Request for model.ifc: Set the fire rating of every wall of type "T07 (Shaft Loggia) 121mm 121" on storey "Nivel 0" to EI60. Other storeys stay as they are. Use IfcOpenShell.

First a look at what the model holds.

```python
import ifcopenshell
import ifcopenshell.util.element

model = ifcopenshell.open("model.ifc")
print(model.schema)
storey = next(s for s in model.by_type("IfcBuildingStorey") if s.Name == "Nivel 0")
walls = [e for e in ifcopenshell.util.element.get_decomposition(storey) if e.is_a("IfcWall")]
seen = {}
for e in walls:
    element_type = ifcopenshell.util.element.get_type(e)
    key = (element_type.Name if element_type != e and element_type else None, ifcopenshell.util.element.get_pset(e, "Pset_WallCommon", "FireRating"))
    seen[key] = seen.get(key, 0) + 1
for (name, value), count in sorted(seen.items(), key=str):
    print(count, "x", name, "|", value)
```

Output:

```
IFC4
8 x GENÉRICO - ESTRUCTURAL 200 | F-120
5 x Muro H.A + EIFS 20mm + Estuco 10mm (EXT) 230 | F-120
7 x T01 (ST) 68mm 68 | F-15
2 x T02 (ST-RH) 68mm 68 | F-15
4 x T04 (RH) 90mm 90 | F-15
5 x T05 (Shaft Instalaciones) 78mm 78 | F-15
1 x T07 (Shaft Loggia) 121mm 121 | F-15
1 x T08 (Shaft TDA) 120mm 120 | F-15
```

```python
import ifcopenshell
import ifcopenshell.api.pset
import ifcopenshell.util.element

model = ifcopenshell.open("model.ifc")

storey = next(s for s in model.by_type("IfcBuildingStorey") if s.Name == "Nivel 0")
walls = [e for e in ifcopenshell.util.element.get_decomposition(storey) if e.is_a("IfcWall")]

count = 0
for e in walls:
    element_type = ifcopenshell.util.element.get_type(e)
    if element_type in (None, e) or element_type.Name != "T07 (Shaft Loggia) 121mm 121":
        continue
    # add_pset returns the element's existing set when there is one.
    pset = ifcopenshell.api.pset.add_pset(model, product=e, name="Pset_WallCommon")
    ifcopenshell.api.pset.edit_pset(model, pset=pset, properties={"FireRating": "EI60"})
    count += 1

print(count, "walls updated")

model.write("model_updated.ifc")
```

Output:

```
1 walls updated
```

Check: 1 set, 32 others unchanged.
